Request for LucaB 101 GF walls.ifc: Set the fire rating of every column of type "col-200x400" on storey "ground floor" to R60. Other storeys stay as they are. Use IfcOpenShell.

First a look at what the model holds.

```python
import ifcopenshell
import ifcopenshell.util.element

model = ifcopenshell.open("LucaB 101 GF walls.ifc")
print(model.schema)
storey = next(s for s in model.by_type("IfcBuildingStorey") if s.Name == "ground floor")
columns = [e for e in ifcopenshell.util.element.get_decomposition(storey) if e.is_a("IfcColumn")]
seen = {}
for e in columns:
    element_type = ifcopenshell.util.element.get_type(e)
    key = (element_type.Name if element_type != e and element_type else None, ifcopenshell.util.element.get_pset(e, "Pset_ColumnCommon", "FireRating"))
    seen[key] = seen.get(key, 0) + 1
for (name, value), count in sorted(seen.items(), key=str):
    print(count, "x", name, "|", value)
```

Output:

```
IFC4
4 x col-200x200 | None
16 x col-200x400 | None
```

```python
import ifcopenshell
import ifcopenshell.api.pset
import ifcopenshell.util.element

model = ifcopenshell.open("LucaB 101 GF walls.ifc")

storey = next(s for s in model.by_type("IfcBuildingStorey") if s.Name == "ground floor")
columns = [e for e in ifcopenshell.util.element.get_decomposition(storey) if e.is_a("IfcColumn")]

count = 0
for e in columns:
    element_type = ifcopenshell.util.element.get_type(e)
    if element_type in (None, e) or element_type.Name != "col-200x400":
        continue
    # add_pset returns the element's existing set when there is one.
    pset = ifcopenshell.api.pset.add_pset(model, product=e, name="Pset_ColumnCommon")
    ifcopenshell.api.pset.edit_pset(model, pset=pset, properties={"FireRating": "R60"})
    count += 1

print(count, "columns updated")

model.write("LucaB 101 GF walls_edited.ifc")
```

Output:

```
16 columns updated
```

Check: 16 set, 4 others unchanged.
